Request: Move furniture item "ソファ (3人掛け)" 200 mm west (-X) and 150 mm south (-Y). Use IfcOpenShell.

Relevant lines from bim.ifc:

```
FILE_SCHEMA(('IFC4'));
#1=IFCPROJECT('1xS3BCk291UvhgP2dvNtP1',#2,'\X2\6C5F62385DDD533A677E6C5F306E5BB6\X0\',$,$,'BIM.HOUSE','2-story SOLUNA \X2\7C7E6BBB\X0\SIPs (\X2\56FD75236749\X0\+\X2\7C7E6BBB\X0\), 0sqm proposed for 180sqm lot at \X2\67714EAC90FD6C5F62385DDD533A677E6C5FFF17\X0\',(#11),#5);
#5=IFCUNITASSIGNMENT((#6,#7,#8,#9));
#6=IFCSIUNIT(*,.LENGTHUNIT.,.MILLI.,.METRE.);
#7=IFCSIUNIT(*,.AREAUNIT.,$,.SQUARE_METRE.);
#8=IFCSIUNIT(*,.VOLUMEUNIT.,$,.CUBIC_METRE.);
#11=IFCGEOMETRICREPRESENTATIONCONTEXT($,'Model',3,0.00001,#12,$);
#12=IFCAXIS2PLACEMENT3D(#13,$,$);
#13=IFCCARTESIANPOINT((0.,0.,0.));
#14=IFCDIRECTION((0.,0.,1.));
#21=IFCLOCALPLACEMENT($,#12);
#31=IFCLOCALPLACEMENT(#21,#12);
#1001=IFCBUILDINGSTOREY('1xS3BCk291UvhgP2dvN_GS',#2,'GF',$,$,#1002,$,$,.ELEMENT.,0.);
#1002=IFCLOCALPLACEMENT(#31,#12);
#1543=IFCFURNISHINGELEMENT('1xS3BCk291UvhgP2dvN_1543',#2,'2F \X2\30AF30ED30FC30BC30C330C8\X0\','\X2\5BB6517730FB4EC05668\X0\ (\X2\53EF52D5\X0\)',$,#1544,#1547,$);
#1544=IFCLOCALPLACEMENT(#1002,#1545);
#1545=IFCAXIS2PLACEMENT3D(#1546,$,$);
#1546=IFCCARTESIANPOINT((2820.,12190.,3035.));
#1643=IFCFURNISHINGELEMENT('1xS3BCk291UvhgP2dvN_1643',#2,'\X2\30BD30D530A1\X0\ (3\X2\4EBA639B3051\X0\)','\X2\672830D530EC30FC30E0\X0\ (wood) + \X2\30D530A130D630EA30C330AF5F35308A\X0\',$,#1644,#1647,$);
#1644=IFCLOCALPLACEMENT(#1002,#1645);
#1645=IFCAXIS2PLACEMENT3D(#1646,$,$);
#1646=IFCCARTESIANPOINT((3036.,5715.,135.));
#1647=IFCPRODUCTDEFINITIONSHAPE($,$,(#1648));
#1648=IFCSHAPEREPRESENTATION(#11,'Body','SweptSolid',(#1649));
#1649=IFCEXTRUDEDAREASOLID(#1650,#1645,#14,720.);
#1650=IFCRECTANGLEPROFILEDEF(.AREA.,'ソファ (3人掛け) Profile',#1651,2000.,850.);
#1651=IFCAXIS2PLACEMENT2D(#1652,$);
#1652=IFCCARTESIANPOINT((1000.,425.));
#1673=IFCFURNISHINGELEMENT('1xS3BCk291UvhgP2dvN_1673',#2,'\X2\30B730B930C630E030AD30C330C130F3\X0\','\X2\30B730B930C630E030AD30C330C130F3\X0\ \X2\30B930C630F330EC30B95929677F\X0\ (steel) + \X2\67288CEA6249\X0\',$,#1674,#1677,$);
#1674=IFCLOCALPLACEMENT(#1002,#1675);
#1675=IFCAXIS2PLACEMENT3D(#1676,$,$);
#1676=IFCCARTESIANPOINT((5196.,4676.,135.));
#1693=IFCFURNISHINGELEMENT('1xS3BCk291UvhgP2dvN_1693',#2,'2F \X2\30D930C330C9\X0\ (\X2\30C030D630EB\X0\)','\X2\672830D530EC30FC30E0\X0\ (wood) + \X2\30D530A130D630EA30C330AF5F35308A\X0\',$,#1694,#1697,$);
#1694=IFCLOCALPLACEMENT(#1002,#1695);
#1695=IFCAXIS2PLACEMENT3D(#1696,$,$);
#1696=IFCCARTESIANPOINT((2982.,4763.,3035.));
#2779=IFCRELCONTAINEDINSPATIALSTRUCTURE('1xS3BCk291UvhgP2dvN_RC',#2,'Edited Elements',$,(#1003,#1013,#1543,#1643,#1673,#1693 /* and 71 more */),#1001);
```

```python
import ifcopenshell
import ifcopenshell.api.geometry
import ifcopenshell.util.placement
import ifcopenshell.util.unit

model = ifcopenshell.open("bim.ifc")
unit_scale = ifcopenshell.util.unit.calculate_unit_scale(model)

item = model.by_id(1643)
matrix = ifcopenshell.util.placement.get_local_placement(item.ObjectPlacement)
matrix[0, 3] -= 0.2 / unit_scale
matrix[1, 3] -= 0.15 / unit_scale
ifcopenshell.api.geometry.edit_object_placement(model, product=item, matrix=matrix, is_si=False)

print(ifcopenshell.util.placement.get_local_placement(item.ObjectPlacement).round(3) + 0.0)

model.write("bim_v2.ifc")
```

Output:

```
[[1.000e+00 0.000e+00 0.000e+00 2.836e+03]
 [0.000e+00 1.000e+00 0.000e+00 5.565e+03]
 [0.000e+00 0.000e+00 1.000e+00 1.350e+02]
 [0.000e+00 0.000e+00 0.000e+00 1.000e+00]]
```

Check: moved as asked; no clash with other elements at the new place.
